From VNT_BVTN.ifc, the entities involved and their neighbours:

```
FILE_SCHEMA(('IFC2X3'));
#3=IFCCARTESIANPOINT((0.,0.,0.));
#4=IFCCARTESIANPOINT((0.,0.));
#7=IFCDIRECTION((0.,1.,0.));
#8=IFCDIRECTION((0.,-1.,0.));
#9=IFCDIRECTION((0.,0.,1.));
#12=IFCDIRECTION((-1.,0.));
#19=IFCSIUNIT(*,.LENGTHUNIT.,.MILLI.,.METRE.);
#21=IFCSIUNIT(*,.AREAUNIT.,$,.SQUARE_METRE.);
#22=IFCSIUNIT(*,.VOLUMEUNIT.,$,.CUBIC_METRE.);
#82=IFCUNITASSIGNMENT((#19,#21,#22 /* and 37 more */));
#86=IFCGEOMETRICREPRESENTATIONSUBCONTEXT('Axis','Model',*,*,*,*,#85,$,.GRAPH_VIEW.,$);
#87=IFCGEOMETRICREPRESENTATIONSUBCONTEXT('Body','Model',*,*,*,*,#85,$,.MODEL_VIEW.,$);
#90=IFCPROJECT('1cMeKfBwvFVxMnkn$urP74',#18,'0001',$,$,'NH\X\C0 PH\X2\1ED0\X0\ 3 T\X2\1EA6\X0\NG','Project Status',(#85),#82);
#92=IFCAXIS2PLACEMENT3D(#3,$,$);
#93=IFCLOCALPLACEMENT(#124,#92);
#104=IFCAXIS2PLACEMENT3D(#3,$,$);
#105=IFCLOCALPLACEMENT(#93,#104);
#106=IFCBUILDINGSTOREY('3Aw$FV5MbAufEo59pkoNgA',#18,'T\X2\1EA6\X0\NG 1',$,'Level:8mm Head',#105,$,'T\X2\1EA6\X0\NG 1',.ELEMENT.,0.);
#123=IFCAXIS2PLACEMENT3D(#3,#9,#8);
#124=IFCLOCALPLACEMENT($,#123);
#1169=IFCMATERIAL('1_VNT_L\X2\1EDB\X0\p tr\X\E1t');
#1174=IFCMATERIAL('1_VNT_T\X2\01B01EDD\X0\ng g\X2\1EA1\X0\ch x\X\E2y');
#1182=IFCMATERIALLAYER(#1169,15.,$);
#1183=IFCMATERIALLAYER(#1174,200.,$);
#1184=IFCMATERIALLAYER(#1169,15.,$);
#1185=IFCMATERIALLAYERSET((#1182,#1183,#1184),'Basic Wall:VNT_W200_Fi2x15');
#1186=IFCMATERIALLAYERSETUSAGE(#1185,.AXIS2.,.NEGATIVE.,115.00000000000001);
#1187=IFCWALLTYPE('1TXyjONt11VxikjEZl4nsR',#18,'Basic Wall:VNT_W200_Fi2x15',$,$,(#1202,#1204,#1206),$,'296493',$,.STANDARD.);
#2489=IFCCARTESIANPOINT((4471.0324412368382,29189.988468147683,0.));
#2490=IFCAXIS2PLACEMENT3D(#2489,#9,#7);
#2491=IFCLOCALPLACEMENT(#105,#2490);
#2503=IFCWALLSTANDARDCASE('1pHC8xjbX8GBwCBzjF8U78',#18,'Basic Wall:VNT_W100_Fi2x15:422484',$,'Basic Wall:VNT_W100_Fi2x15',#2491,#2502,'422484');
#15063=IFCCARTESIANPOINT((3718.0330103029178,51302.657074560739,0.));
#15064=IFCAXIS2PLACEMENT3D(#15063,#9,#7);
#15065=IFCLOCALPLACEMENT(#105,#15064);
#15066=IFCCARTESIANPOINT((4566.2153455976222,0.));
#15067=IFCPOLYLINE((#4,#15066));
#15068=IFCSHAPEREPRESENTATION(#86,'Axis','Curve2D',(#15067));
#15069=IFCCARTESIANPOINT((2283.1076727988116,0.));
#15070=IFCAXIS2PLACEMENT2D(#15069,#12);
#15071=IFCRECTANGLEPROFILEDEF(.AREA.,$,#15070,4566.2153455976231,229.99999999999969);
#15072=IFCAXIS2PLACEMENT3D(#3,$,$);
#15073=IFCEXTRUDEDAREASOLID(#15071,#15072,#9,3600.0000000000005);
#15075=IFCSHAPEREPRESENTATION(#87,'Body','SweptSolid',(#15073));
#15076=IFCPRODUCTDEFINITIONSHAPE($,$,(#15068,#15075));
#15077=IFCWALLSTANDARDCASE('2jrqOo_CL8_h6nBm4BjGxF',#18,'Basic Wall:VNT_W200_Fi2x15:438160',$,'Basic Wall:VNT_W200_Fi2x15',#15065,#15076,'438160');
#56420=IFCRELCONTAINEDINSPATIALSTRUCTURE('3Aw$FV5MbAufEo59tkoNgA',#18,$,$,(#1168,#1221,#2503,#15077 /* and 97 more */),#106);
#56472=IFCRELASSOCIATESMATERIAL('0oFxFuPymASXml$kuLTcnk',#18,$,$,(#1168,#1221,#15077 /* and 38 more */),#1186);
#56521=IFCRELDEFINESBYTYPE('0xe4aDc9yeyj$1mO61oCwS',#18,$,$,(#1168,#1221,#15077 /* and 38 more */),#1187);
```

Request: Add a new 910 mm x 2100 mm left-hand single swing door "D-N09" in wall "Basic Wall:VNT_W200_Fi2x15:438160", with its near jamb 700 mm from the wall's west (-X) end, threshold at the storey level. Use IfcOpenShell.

```python
import numpy as np
import ifcopenshell
import ifcopenshell.api.feature
import ifcopenshell.api.geometry
import ifcopenshell.api.root
import ifcopenshell.api.spatial
import ifcopenshell.api.type
import ifcopenshell.geom
import ifcopenshell.util.element
import ifcopenshell.util.placement
import ifcopenshell.util.representation
import ifcopenshell.util.shape
import ifcopenshell.util.unit

model = ifcopenshell.open("VNT_BVTN.ifc")
unit_scale = ifcopenshell.util.unit.calculate_unit_scale(model)
settings = ifcopenshell.geom.settings()


def volume(element):
    """Net volume in cubic metres, openings subtracted."""
    shape = ifcopenshell.geom.create_shape(settings, element)
    return ifcopenshell.util.shape.get_volume(shape.geometry)


wall = model.by_guid("2jrqOo_CL8_h6nBm4BjGxF")
storey = ifcopenshell.util.element.get_container(wall, ifc_class="IfcBuildingStorey")
context = ifcopenshell.util.representation.get_context(model, "Model", "Body", "MODEL_VIEW")
before = volume(wall)

width, height, from_end, sill = 0.91, 2.1, 0.7, 0.0  # metres

# The wall runs along its own X axis, and the end named is its -X end.
wall_shape = ifcopenshell.geom.create_shape(settings, wall)
x, y, z = ifcopenshell.util.shape.get_vertices(wall_shape.geometry).T
start = x.min() + from_end
face, thickness = float(y.min()), float(y.max() - y.min())
wall_matrix = ifcopenshell.util.placement.get_local_placement(wall.ObjectPlacement)
level = ifcopenshell.util.placement.get_local_placement(storey.ObjectPlacement)[2, 3]


def in_wall(x, y):
    """Placement at x, y metres in the wall's axes, at sill height."""
    matrix = wall_matrix.copy()
    matrix[:, 3] = wall_matrix @ np.array([x / unit_scale, y / unit_scale, 0.0, 1.0])
    matrix[2, 3] = level + sill / unit_scale
    return matrix


# Opening: a box that overshoots both wall faces by 50 mm.
opening = ifcopenshell.api.root.create_entity(model, ifc_class="IfcOpeningElement")
box = ifcopenshell.api.geometry.add_wall_representation(
    model, context=context, length=width, height=height, thickness=thickness + 0.1
)
ifcopenshell.api.geometry.assign_representation(model, product=opening, representation=box)
ifcopenshell.api.geometry.edit_object_placement(model, product=opening, matrix=in_wall(start, face - 0.05), is_si=False)
ifcopenshell.api.feature.add_feature(model, feature=opening, element=wall)

door = ifcopenshell.api.root.create_entity(model, ifc_class="IfcDoor", name="D-N09")
door.OverallWidth, door.OverallHeight = width / unit_scale, height / unit_scale
body = ifcopenshell.api.geometry.add_door_representation(
    model,
    context=context,
    overall_width=door.OverallWidth,
    overall_height=door.OverallHeight,
    operation_type="SINGLE_SWING_LEFT",
    lining_properties={"LiningDepth": thickness / unit_scale, "ThresholdDepth": thickness / unit_scale},
)
ifcopenshell.api.geometry.assign_representation(model, product=door, representation=body)
ifcopenshell.api.spatial.assign_container(model, products=[door], relating_structure=storey)
fills = ifcopenshell.api.feature.add_filling(model, opening=opening, element=door)
fills.OwnerHistory = door.OwnerHistory  # required in IFC2X3

# IFC2X3 keeps the operation on the door style.
style = ifcopenshell.api.root.create_entity(model, ifc_class="IfcDoorStyle", name="D-N09")
style.OperationType, style.ConstructionType = "SINGLE_SWING_LEFT", "NOTDEFINED"
style.ParameterTakesPrecedence = style.Sizeable = False
ifcopenshell.api.type.assign_type(model, related_objects=[door], relating_type=style)

# The lining spans the wall, so the door starts at the wall face.
ifcopenshell.api.geometry.edit_object_placement(model, product=door, matrix=in_wall(start, face), is_si=False)

after = volume(wall)

print(f"wall volume {before:.3f} -> {after:.3f} m3")

model.write("VNT_BVTN_v2.ifc")
```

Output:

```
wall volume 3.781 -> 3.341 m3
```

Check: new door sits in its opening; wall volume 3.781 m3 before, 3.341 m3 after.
